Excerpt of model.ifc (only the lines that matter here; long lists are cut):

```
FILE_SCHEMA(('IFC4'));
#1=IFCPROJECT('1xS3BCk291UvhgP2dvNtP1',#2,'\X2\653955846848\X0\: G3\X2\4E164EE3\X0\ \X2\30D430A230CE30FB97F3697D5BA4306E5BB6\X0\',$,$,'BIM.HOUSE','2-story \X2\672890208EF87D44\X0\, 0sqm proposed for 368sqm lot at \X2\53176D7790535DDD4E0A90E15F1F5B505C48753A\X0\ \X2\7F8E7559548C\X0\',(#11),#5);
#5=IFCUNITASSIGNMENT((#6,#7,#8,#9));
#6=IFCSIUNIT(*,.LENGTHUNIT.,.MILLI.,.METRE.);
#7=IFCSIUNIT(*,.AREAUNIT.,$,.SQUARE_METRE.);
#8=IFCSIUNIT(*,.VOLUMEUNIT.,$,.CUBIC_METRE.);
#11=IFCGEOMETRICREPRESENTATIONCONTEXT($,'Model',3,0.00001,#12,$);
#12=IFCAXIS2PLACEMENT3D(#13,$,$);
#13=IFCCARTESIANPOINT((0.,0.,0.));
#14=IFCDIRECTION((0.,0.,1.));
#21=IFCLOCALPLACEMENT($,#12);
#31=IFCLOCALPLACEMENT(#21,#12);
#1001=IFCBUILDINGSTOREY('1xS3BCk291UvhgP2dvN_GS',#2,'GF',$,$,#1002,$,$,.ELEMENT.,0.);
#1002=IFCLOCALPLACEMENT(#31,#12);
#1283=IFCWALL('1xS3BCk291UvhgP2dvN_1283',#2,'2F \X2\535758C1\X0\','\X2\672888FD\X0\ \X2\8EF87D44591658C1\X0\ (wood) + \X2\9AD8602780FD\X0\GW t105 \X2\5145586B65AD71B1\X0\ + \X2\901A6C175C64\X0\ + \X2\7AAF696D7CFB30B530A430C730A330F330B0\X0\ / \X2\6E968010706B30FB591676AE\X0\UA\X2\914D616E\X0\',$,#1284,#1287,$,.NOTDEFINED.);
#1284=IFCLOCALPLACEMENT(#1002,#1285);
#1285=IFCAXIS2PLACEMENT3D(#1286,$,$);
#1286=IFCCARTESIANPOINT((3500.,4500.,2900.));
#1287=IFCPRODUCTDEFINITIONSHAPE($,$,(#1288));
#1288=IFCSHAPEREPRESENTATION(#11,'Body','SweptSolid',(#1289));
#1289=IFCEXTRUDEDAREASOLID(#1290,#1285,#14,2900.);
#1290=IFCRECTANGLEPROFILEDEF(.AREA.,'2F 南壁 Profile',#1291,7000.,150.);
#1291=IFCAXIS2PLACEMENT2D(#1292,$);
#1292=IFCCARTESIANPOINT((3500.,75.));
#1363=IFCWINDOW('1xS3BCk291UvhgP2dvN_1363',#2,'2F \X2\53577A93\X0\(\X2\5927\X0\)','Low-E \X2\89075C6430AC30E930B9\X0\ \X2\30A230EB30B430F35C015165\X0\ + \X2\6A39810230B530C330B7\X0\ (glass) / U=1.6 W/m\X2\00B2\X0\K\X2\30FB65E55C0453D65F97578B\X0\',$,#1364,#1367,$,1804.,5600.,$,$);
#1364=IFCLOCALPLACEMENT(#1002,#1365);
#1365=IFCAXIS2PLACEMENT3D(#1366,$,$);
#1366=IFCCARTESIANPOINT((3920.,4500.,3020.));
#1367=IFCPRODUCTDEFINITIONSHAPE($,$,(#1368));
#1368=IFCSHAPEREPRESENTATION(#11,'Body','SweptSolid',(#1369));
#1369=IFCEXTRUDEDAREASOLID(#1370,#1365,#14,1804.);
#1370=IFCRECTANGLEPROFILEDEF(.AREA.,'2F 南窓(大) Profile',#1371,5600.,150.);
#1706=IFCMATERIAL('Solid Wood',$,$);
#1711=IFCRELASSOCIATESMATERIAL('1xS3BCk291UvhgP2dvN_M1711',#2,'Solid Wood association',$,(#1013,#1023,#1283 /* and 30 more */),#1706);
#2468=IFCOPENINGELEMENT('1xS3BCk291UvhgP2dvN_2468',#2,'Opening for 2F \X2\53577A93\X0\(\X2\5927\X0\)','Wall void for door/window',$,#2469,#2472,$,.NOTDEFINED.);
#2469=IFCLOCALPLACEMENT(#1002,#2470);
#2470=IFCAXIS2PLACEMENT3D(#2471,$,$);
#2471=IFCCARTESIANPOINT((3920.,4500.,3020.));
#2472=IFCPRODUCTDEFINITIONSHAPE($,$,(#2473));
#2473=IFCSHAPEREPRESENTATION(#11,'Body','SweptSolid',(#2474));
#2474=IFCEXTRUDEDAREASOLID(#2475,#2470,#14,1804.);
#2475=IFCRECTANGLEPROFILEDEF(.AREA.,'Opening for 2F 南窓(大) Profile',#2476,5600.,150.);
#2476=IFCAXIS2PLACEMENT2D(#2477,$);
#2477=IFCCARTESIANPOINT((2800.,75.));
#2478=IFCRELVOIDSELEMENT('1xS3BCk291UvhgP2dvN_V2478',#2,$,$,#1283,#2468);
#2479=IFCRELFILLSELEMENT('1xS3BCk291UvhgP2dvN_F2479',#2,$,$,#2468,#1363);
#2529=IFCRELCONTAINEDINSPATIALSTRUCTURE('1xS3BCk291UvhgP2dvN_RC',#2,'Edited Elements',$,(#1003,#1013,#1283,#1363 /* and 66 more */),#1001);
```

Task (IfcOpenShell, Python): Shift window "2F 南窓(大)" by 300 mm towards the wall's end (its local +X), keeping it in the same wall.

```python
import ifcopenshell
import ifcopenshell.api.geometry
import ifcopenshell.util.placement

model = ifcopenshell.open("model.ifc")

window = model.by_id(1363)
opening = window.FillsVoids[0].RelatingOpeningElement
wall = opening.VoidsElements[0].RelatingBuildingElement

wall_matrix = ifcopenshell.util.placement.get_local_placement(wall.ObjectPlacement)
shift = wall_matrix[:3, 0] * 300.0
before = ifcopenshell.util.placement.get_local_placement(window.ObjectPlacement)[:3, 3].copy()

# The window is not placed relative to its opening, so move both.
for product in (opening, window):
    matrix = ifcopenshell.util.placement.get_local_placement(product.ObjectPlacement)
    matrix[:3, 3] += shift
    ifcopenshell.api.geometry.edit_object_placement(model, product=product, matrix=matrix, is_si=False)

after = ifcopenshell.util.placement.get_local_placement(window.ObjectPlacement)[:3, 3]
print("window moved by", (after - before).round(3) + 0.0)

model.write("model_updated.ifc")
```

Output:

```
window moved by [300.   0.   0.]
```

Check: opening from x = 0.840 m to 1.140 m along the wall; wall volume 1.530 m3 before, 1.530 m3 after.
